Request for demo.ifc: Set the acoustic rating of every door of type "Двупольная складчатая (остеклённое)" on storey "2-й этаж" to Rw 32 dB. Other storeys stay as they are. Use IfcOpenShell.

First a look at what the model holds.

```python
import ifcopenshell
import ifcopenshell.util.element

model = ifcopenshell.open("demo.ifc")
print(model.schema)
storey = next(s for s in model.by_type("IfcBuildingStorey") if s.Name == "2-й этаж")
doors = [e for e in ifcopenshell.util.element.get_decomposition(storey) if e.is_a("IfcDoor")]
seen = {}
for e in doors:
    element_type = ifcopenshell.util.element.get_type(e)
    key = (element_type.Name if element_type != e and element_type else None, ifcopenshell.util.element.get_pset(e, "Pset_DoorCommon", "AcousticRating"))
    seen[key] = seen.get(key, 0) + 1
for (name, value), count in sorted(seen.items(), key=str):
    print(count, "x", name, "|", value)
```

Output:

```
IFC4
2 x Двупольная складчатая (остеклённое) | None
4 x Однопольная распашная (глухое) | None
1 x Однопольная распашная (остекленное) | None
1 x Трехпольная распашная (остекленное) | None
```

```python
import ifcopenshell
import ifcopenshell.api.pset
import ifcopenshell.util.element

model = ifcopenshell.open("demo.ifc")

storey = next(s for s in model.by_type("IfcBuildingStorey") if s.Name == "2-й этаж")
doors = [e for e in ifcopenshell.util.element.get_decomposition(storey) if e.is_a("IfcDoor")]

count = 0
for e in doors:
    element_type = ifcopenshell.util.element.get_type(e)
    if element_type in (None, e) or element_type.Name != "Двупольная складчатая (остеклённое)":
        continue
    # add_pset returns the element's existing set when there is one.
    pset = ifcopenshell.api.pset.add_pset(model, product=e, name="Pset_DoorCommon")
    ifcopenshell.api.pset.edit_pset(model, pset=pset, properties={"AcousticRating": "Rw 32 dB"})
    count += 1

print(count, "doors updated")

model.write("demo-out.ifc")
```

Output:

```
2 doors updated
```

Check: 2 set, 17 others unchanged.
